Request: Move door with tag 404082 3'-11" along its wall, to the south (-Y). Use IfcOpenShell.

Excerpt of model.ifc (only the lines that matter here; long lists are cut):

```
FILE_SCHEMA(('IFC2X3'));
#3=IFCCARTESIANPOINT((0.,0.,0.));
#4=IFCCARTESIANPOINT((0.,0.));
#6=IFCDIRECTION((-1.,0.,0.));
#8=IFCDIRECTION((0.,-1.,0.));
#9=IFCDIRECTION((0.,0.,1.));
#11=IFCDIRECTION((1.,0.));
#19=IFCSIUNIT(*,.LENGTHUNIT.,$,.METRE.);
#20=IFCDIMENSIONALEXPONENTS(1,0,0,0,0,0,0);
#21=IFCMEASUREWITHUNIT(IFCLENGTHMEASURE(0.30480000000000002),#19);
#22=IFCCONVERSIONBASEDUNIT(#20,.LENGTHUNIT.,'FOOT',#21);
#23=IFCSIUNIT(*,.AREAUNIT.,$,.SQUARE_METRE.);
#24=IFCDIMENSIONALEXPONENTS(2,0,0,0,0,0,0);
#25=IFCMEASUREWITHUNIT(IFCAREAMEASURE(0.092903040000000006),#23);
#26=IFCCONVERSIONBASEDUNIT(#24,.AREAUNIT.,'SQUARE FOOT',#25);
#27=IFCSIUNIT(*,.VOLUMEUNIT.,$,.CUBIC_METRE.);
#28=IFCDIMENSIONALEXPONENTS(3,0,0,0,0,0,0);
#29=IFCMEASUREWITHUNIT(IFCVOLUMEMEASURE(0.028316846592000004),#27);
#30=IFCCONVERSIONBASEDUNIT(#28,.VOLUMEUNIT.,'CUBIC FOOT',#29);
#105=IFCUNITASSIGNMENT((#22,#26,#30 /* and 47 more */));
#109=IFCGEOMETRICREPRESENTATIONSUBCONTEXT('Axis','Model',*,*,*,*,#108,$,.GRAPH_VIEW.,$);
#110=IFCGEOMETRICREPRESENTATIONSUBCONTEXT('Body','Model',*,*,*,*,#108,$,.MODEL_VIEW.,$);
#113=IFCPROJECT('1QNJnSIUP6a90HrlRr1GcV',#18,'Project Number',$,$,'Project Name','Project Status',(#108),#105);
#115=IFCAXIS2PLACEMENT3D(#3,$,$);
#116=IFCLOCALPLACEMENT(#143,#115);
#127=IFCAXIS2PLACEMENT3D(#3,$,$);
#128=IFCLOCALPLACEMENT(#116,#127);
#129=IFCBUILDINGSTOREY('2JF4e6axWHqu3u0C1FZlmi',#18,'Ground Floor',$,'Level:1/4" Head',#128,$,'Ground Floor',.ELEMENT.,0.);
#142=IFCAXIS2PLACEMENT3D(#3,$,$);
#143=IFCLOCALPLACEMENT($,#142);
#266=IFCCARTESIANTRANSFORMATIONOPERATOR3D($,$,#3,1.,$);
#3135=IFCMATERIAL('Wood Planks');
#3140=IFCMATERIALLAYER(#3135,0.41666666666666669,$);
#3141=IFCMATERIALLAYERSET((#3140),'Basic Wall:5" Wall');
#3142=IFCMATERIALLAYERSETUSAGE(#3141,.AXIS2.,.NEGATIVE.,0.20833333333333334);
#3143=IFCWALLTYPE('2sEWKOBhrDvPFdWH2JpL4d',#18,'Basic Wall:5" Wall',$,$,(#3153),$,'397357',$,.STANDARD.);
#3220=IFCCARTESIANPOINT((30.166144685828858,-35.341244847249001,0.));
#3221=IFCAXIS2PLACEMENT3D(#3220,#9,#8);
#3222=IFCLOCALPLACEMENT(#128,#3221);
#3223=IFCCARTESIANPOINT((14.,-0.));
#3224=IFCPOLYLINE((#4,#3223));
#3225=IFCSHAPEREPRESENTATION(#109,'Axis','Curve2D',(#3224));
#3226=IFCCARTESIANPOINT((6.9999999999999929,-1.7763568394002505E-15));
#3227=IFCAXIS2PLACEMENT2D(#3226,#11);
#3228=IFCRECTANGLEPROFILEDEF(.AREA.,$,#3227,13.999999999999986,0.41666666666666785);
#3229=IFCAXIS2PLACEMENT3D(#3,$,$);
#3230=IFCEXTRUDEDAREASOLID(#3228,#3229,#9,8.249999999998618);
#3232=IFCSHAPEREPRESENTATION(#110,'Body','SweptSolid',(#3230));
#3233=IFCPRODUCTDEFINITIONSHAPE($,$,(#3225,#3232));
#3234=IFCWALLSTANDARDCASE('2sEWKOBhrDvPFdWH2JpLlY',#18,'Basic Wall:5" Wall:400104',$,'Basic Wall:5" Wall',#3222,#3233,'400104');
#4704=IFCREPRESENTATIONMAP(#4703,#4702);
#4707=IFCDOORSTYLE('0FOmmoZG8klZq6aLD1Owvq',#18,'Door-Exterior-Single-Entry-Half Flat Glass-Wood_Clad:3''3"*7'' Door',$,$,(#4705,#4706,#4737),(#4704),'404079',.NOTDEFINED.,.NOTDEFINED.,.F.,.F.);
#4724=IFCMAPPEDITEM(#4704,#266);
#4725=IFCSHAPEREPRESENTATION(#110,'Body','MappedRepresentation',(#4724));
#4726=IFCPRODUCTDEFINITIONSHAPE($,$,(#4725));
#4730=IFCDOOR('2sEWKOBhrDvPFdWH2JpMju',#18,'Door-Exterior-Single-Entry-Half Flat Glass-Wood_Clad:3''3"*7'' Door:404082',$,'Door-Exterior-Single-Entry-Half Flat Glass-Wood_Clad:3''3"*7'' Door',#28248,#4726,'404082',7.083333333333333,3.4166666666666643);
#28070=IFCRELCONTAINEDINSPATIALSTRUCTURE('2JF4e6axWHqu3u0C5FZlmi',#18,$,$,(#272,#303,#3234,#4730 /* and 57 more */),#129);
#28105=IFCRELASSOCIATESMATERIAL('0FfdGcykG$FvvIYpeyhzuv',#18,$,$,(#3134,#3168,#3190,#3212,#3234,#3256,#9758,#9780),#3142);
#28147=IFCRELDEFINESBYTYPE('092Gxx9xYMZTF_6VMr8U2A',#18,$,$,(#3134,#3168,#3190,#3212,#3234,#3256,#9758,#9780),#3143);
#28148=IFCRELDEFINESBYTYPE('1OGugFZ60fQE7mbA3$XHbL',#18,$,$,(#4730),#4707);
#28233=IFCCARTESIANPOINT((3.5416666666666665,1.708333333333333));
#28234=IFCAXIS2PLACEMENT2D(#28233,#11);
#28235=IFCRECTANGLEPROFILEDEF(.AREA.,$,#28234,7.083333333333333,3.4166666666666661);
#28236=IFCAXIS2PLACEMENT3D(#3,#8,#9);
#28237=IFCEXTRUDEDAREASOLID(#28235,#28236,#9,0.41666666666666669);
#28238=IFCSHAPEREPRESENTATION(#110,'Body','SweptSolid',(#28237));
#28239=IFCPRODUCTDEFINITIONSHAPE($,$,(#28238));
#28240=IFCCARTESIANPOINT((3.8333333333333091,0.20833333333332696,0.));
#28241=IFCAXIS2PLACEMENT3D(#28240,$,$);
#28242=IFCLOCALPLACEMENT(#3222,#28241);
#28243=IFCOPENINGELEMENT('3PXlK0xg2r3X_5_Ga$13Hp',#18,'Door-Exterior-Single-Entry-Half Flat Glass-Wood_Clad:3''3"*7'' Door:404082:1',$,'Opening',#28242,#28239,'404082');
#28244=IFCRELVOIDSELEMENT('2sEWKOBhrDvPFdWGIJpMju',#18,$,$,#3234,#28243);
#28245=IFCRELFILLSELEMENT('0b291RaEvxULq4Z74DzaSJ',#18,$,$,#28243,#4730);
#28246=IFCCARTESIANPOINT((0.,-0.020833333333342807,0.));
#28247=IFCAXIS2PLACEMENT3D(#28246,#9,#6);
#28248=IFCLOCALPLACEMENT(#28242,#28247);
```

```python
import ifcopenshell
import ifcopenshell.api.geometry
import ifcopenshell.util.placement
import ifcopenshell.util.unit

model = ifcopenshell.open("model.ifc")
unit_scale = ifcopenshell.util.unit.calculate_unit_scale(model)

door = model.by_guid("2sEWKOBhrDvPFdWH2JpMju")
opening = door.FillsVoids[0].RelatingOpeningElement
wall = opening.VoidsElements[0].RelatingBuildingElement

wall_matrix = ifcopenshell.util.placement.get_local_placement(wall.ObjectPlacement)
shift = wall_matrix[:3, 0] * 47 * 0.0254 / unit_scale
before = ifcopenshell.util.placement.get_local_placement(door.ObjectPlacement)[:3, 3].copy()

# The door is placed relative to its opening, so it follows when the opening moves.
matrix = ifcopenshell.util.placement.get_local_placement(opening.ObjectPlacement)
matrix[:3, 3] += shift
ifcopenshell.api.geometry.edit_object_placement(
    model, product=opening, matrix=matrix, is_si=False, should_transform_children=True
)

after = ifcopenshell.util.placement.get_local_placement(door.ObjectPlacement)[:3, 3]
print("door moved by", (after - before).round(3) + 0.0)

model.write("model_updated.ifc")
```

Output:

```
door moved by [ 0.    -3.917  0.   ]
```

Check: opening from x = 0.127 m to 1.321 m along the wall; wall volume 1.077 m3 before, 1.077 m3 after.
